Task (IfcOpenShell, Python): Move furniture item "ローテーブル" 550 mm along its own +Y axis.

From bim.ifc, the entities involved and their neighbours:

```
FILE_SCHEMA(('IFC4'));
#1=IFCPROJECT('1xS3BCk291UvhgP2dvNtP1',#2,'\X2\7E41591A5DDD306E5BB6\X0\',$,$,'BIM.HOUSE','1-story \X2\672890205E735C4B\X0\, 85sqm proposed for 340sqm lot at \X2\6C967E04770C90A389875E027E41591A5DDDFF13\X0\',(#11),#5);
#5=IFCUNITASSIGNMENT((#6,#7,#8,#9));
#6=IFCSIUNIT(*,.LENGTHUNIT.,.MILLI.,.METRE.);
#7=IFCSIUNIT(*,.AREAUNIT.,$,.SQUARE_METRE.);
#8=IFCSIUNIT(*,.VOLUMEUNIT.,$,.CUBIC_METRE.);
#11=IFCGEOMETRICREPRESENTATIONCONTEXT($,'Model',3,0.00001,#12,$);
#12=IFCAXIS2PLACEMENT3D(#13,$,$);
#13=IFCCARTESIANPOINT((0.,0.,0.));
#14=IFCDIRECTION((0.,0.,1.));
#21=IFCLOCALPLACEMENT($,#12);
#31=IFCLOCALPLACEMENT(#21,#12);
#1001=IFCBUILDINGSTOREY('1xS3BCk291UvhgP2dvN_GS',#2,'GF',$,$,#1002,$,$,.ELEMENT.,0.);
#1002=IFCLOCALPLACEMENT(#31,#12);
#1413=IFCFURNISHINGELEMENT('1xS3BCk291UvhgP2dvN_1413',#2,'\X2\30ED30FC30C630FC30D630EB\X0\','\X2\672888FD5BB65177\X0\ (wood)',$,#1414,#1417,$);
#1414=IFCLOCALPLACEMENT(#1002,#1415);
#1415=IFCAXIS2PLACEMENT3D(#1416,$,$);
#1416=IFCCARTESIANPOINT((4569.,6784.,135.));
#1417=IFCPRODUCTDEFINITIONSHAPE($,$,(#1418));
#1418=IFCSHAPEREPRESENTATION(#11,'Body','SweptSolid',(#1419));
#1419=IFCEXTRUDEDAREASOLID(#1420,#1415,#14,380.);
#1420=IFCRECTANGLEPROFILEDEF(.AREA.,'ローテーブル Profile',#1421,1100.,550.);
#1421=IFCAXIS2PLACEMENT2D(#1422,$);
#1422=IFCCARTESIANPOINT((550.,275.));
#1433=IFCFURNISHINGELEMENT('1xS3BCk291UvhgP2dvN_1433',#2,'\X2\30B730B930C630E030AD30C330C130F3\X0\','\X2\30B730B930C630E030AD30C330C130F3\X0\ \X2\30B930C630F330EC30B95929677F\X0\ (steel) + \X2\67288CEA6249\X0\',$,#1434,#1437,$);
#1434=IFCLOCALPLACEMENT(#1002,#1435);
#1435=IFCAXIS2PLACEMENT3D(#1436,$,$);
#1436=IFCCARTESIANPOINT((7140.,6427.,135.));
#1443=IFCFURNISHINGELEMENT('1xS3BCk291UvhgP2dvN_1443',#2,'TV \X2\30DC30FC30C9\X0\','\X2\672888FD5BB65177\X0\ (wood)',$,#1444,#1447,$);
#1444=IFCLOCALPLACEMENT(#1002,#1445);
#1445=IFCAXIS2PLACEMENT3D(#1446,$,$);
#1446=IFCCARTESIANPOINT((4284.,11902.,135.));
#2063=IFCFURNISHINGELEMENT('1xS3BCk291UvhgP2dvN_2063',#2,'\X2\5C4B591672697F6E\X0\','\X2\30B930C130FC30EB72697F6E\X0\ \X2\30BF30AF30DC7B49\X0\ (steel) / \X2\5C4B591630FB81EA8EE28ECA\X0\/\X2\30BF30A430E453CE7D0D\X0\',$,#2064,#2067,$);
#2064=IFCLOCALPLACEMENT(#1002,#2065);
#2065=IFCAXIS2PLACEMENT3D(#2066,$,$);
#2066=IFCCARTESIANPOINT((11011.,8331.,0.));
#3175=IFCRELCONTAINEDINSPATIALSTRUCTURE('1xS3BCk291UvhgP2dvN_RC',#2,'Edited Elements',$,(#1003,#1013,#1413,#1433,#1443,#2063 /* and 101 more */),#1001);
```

```python
import ifcopenshell
import ifcopenshell.api.geometry
import ifcopenshell.util.placement

model = ifcopenshell.open("bim.ifc")

item = model.by_guid("1xS3BCk291UvhgP2dvN_1413")
matrix = ifcopenshell.util.placement.get_local_placement(item.ObjectPlacement)
matrix[:3, 3] += matrix[:3, 1] * 550.0
ifcopenshell.api.geometry.edit_object_placement(model, product=item, matrix=matrix, is_si=False)

print(ifcopenshell.util.placement.get_local_placement(item.ObjectPlacement).round(3) + 0.0)

model.write("bim_v2.ifc")
```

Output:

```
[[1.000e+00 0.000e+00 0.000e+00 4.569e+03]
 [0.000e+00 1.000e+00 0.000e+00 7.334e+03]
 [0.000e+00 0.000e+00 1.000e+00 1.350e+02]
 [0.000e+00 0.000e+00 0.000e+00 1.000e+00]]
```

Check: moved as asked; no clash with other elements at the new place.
